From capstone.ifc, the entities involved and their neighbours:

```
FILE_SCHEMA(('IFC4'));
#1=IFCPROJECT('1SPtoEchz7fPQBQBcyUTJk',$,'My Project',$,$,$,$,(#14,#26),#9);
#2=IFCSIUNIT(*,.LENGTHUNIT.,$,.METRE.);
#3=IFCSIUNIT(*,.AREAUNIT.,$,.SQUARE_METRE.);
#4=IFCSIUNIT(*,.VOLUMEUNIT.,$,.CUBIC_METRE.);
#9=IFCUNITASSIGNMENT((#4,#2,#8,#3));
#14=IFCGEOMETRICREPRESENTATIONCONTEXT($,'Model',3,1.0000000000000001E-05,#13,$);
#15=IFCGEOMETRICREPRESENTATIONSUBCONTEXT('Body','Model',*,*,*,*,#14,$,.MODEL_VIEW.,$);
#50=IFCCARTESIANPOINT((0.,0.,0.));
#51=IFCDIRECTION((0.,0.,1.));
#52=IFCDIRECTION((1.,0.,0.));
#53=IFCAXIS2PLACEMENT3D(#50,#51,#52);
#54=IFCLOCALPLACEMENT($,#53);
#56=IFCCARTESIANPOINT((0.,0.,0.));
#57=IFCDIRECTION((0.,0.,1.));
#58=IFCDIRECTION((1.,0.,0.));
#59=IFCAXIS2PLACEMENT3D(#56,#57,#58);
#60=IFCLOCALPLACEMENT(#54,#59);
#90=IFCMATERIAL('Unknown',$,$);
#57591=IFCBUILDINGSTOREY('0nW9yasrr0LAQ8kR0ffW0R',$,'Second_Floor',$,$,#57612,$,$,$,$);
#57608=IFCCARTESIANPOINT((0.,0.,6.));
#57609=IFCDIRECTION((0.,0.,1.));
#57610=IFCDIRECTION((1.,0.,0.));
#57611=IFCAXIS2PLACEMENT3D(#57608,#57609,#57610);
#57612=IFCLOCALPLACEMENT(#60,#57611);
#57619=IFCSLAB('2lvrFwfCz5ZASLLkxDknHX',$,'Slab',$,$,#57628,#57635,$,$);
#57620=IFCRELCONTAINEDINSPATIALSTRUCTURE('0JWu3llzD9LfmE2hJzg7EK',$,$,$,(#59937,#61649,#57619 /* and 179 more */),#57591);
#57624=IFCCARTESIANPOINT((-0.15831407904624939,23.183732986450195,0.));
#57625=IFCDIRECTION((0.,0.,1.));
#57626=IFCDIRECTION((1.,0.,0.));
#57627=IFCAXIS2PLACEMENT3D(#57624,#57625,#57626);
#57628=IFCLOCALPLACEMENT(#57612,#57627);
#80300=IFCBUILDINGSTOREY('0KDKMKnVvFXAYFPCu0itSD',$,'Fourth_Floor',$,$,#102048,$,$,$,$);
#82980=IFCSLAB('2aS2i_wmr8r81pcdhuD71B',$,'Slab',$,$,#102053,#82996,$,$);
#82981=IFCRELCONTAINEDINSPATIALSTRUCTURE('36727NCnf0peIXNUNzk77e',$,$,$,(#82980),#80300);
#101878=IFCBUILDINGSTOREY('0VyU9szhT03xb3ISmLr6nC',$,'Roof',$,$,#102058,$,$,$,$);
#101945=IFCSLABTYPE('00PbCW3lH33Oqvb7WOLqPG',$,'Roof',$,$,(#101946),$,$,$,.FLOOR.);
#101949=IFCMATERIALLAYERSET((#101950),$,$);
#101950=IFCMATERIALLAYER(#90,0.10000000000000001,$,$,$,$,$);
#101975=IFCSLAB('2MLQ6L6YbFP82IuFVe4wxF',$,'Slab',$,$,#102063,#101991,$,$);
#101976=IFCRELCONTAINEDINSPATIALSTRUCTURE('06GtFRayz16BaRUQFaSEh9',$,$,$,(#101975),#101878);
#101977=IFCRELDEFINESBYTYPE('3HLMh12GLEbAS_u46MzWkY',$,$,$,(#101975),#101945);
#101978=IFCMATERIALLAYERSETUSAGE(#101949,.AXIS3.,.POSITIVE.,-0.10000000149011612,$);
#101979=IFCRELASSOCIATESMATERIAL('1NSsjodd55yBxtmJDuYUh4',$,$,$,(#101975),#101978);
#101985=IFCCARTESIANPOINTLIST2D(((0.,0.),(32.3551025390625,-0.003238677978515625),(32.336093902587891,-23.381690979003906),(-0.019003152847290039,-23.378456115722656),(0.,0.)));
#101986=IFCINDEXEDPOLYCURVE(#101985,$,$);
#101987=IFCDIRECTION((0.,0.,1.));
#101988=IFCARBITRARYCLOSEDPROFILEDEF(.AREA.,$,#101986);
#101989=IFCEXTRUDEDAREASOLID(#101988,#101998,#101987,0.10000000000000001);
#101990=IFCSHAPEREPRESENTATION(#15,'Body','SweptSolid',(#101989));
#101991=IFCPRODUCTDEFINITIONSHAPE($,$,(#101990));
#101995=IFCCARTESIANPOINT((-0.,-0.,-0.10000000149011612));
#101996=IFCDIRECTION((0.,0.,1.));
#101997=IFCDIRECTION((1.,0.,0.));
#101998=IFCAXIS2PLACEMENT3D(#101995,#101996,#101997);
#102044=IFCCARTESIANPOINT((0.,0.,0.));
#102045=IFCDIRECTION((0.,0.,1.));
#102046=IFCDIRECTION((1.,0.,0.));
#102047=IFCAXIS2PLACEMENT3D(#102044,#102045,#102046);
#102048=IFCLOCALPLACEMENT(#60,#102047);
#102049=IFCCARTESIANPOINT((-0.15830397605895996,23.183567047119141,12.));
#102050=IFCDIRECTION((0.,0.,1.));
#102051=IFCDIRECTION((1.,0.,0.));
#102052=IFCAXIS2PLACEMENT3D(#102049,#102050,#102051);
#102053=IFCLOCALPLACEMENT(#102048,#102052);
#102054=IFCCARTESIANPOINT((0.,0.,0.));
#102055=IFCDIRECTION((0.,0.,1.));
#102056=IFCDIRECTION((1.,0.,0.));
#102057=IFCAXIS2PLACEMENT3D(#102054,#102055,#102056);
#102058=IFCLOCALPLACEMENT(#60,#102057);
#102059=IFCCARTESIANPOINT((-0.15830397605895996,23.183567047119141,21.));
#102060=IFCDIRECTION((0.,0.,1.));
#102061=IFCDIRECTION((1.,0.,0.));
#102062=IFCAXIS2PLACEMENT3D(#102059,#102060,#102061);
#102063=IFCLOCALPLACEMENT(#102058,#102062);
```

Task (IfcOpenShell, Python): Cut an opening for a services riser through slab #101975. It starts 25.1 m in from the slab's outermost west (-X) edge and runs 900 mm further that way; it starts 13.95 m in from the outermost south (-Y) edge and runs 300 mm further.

```python
import numpy as np
import ifcopenshell
import ifcopenshell.api.feature
import ifcopenshell.api.geometry
import ifcopenshell.api.root
import ifcopenshell.geom
import ifcopenshell.util.placement
import ifcopenshell.util.representation
import ifcopenshell.util.shape
import ifcopenshell.util.unit

model = ifcopenshell.open("capstone.ifc")
unit_scale = ifcopenshell.util.unit.calculate_unit_scale(model)
settings = ifcopenshell.geom.settings()


def volume(element):
    """Net volume in cubic metres, openings subtracted."""
    shape = ifcopenshell.geom.create_shape(settings, element)
    return ifcopenshell.util.shape.get_volume(shape.geometry)


slab = model.by_guid("2MLQ6L6YbFP82IuFVe4wxF")
before = volume(slab)

# Extent in the slab's own axes, in metres. The edges named are its -X and -Y sides.
slab_shape = ifcopenshell.geom.create_shape(settings, slab)
vertices = ifcopenshell.util.shape.get_vertices(slab_shape.geometry)
x_min, y_min, bottom = vertices.min(axis=0)
top = vertices[:, 2].max()

opening = ifcopenshell.api.root.create_entity(model, ifc_class="IfcOpeningElement", name="Services riser opening", predefined_type="OPENING")
context = ifcopenshell.util.representation.get_context(model, "Model", "Body", "MODEL_VIEW")
width, depth = 0.9, 0.3
outline = [(0.0, 0.0), (width, 0.0), (width, depth), (0.0, depth), (0.0, 0.0)]
# Overshoot both faces by 50 mm so the cut is clean.
shape = ifcopenshell.api.geometry.add_slab_representation(
    model, context=context, depth=top - bottom + 0.1, polyline=outline
)
ifcopenshell.api.geometry.assign_representation(model, product=opening, representation=shape)

matrix = ifcopenshell.util.placement.get_local_placement(slab.ObjectPlacement)
matrix[:, 3] = matrix @ np.append(np.array([x_min + 25.1, y_min + 13.95, bottom - 0.05]) / unit_scale, 1.0)
ifcopenshell.api.geometry.edit_object_placement(model, product=opening, matrix=matrix, is_si=False)
ifcopenshell.api.feature.add_feature(model, feature=opening, element=slab)

after = volume(slab)

print(f"slab volume {before:.3f} -> {after:.3f} m3")

model.write("capstone_v2.ifc")
```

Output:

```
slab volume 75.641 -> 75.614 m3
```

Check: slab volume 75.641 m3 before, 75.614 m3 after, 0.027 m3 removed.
